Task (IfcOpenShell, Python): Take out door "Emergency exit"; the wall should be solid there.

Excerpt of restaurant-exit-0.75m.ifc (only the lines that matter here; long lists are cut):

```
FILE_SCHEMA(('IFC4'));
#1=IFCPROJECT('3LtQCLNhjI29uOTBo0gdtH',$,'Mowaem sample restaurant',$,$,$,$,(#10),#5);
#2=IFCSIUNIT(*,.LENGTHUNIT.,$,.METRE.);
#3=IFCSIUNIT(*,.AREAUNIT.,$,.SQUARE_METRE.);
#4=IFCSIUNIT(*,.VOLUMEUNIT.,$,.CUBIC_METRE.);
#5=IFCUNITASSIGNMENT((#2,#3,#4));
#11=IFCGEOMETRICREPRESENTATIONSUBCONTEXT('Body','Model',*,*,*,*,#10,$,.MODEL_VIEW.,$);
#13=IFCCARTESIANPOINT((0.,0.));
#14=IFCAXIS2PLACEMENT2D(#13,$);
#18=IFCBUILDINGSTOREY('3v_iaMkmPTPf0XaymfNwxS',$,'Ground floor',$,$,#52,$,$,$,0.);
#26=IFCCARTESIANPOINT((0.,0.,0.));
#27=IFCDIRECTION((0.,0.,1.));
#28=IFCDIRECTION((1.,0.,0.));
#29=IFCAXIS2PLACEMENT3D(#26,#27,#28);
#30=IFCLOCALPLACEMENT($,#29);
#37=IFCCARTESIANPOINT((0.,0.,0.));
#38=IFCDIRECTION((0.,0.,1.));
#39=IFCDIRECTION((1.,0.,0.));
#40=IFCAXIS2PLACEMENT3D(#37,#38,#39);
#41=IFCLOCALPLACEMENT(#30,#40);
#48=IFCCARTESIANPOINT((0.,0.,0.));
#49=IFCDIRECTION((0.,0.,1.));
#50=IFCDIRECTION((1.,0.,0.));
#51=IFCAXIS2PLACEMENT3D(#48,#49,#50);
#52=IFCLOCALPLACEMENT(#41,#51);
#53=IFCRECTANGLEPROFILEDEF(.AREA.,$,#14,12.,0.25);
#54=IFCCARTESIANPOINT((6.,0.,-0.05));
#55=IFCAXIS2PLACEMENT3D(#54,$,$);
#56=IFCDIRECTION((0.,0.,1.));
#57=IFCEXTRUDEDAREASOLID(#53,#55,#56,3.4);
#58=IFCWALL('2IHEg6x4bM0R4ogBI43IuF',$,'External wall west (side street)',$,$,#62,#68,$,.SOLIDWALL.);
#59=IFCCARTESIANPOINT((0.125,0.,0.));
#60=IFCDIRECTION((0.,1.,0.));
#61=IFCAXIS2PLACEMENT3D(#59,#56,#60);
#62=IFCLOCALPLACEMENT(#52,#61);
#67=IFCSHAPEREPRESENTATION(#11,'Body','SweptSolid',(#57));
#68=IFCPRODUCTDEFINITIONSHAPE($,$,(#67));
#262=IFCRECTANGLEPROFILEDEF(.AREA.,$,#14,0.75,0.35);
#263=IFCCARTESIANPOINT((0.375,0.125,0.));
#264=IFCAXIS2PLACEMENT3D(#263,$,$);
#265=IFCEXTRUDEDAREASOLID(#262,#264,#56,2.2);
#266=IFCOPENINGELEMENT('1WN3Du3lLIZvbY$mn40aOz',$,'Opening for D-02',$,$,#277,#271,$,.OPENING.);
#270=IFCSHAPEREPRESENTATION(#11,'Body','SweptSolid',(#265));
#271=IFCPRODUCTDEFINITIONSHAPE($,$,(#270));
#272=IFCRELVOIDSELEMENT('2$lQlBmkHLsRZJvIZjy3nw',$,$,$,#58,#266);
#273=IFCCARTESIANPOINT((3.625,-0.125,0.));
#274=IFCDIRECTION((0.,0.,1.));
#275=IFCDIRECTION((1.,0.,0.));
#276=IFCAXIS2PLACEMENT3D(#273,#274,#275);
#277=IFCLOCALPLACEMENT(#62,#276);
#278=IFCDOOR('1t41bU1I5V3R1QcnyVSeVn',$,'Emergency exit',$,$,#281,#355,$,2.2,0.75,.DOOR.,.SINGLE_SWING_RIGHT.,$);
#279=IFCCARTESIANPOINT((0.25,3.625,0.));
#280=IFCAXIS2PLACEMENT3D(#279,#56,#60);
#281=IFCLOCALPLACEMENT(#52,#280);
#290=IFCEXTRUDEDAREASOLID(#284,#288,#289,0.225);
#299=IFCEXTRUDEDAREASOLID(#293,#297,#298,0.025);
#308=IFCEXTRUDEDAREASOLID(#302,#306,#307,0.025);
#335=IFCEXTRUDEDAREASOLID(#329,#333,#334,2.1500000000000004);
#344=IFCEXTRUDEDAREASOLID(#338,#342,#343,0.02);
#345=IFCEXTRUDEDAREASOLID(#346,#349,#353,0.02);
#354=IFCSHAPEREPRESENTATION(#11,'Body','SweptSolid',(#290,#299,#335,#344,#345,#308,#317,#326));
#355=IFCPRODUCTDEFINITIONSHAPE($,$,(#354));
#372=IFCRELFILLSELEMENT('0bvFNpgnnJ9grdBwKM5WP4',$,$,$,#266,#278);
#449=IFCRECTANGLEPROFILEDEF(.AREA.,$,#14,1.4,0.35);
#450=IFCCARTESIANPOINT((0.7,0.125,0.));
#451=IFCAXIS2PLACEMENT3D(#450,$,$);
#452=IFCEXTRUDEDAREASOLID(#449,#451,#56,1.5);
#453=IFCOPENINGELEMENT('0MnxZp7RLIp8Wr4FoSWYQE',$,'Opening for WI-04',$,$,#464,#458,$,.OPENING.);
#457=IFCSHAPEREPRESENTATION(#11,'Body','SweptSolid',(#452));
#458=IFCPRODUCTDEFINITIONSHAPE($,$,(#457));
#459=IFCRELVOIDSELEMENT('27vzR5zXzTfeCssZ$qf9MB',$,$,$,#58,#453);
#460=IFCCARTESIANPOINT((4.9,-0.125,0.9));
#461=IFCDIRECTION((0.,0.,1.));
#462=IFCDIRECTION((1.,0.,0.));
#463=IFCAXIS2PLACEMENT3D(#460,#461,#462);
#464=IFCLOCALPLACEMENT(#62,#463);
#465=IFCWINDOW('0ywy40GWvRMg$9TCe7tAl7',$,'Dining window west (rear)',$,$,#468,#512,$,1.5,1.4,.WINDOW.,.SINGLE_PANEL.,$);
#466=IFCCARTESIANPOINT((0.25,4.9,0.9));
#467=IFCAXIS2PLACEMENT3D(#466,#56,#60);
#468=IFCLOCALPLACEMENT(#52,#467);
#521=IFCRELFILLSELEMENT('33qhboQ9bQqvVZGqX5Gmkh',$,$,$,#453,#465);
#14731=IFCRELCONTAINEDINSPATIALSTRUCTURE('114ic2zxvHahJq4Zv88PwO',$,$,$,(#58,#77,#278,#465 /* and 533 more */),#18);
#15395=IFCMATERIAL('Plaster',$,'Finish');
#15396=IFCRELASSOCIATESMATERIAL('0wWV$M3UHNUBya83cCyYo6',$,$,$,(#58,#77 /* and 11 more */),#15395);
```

```python
import ifcopenshell
import ifcopenshell.api.feature
import ifcopenshell.api.root
import ifcopenshell.geom
import ifcopenshell.util.shape

model = ifcopenshell.open("restaurant-exit-0.75m.ifc")
settings = ifcopenshell.geom.settings()


def volume(element):
    """Net volume in cubic metres, openings subtracted."""
    shape = ifcopenshell.geom.create_shape(settings, element)
    return ifcopenshell.util.shape.get_volume(shape.geometry)


door = model.by_guid("1t41bU1I5V3R1QcnyVSeVn")
opening = door.FillsVoids[0].RelatingOpeningElement
wall = opening.VoidsElements[0].RelatingBuildingElement
before = volume(wall)

ifcopenshell.api.root.remove_product(model, product=door)
ifcopenshell.api.feature.remove_feature(model, feature=opening)

after = volume(wall)

print(f"wall volume {before:.3f} -> {after:.3f} m3")

model.write("restaurant-exit-0.75m_v2.ifc")
```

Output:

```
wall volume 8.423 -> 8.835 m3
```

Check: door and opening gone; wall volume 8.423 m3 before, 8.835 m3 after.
